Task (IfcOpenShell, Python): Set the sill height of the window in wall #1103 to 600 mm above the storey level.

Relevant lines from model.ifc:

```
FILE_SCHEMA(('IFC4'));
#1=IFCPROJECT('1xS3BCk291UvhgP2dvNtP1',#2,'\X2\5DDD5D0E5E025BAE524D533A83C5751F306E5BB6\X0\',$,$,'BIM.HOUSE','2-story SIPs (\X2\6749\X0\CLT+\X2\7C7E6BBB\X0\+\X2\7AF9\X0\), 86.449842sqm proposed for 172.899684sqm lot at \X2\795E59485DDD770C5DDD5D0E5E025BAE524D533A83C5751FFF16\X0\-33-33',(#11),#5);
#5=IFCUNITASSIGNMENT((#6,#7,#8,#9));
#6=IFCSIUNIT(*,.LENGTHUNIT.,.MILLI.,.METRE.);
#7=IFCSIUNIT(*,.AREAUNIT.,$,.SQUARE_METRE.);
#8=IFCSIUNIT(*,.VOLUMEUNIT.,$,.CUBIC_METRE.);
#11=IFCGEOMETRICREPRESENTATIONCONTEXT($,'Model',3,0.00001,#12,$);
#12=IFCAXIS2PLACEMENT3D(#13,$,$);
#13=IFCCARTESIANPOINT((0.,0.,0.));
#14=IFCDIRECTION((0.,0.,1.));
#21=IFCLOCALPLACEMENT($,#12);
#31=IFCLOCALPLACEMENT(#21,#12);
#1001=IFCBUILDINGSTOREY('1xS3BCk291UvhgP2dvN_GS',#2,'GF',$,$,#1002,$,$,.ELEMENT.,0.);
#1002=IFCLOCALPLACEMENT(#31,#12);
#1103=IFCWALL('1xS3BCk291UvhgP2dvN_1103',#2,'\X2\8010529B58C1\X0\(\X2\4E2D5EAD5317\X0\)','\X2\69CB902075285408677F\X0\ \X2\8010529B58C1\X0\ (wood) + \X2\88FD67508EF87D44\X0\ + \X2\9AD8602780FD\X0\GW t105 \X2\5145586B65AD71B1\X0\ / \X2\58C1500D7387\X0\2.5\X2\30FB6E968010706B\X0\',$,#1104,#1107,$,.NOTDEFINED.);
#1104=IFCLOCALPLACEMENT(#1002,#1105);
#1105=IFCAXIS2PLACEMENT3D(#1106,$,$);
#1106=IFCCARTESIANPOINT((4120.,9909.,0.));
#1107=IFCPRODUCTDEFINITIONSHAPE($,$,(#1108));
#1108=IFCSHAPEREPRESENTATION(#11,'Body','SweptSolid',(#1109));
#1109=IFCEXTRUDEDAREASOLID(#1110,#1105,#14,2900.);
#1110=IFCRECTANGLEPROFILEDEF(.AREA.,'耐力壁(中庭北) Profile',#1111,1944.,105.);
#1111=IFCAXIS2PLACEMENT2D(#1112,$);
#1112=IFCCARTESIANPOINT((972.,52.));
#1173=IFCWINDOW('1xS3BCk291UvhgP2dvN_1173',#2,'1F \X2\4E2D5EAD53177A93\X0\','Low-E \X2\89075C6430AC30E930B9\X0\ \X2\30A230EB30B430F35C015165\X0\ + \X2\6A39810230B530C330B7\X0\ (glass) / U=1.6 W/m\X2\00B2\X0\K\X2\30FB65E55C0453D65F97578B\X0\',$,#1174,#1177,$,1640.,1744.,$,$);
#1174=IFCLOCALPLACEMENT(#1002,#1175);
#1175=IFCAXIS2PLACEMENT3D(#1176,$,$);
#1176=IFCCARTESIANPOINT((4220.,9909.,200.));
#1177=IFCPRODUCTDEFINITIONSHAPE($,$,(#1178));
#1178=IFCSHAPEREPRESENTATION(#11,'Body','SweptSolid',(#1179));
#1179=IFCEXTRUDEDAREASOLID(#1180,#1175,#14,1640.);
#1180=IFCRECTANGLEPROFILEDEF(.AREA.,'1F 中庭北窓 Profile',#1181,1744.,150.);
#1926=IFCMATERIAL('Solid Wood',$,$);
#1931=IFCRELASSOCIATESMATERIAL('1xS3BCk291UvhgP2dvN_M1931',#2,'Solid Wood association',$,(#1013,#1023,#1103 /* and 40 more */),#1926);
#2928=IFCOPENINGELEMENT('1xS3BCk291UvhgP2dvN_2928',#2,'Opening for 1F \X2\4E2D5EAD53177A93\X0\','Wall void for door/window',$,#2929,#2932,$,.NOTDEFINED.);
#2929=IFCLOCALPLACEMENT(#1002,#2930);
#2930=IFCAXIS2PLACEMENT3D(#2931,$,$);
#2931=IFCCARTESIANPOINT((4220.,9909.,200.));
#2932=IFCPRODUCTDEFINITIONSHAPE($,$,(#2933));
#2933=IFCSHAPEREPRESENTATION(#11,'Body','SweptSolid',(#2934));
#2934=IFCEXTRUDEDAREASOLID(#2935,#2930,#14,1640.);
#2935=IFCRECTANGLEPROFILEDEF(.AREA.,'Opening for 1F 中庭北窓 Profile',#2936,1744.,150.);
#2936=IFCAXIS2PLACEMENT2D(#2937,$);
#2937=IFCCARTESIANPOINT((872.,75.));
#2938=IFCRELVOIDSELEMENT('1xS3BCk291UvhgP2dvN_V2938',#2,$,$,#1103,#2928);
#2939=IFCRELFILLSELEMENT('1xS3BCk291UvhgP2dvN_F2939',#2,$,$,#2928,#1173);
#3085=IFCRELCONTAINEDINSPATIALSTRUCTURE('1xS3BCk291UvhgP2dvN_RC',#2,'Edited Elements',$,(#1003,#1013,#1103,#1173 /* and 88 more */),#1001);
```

```python
import numpy as np
import ifcopenshell
import ifcopenshell.api.geometry
import ifcopenshell.geom
import ifcopenshell.util.element
import ifcopenshell.util.placement
import ifcopenshell.util.shape
import ifcopenshell.util.unit

model = ifcopenshell.open("model.ifc")
unit_scale = ifcopenshell.util.unit.calculate_unit_scale(model)

window = model.by_guid("1xS3BCk291UvhgP2dvN_1173")
opening = window.FillsVoids[0].RelatingOpeningElement
storey = ifcopenshell.util.element.get_container(window, ifc_class="IfcBuildingStorey")
level = ifcopenshell.util.placement.get_local_placement(storey.ObjectPlacement)[2, 3]

# The opening's origin need not be at the sill, so measure its lowest point.
shape = ifcopenshell.geom.create_shape(ifcopenshell.geom.settings(), opening)
bottom = ifcopenshell.util.shape.get_shape_bottom_elevation(shape, shape.geometry) / unit_scale
dz = level + 600.0 - bottom

shift = np.array([0.0, 0.0, dz])
# The window is not placed relative to its opening, so move both.
for product in (opening, window):
    matrix = ifcopenshell.util.placement.get_local_placement(product.ObjectPlacement)
    matrix[:3, 3] += shift
    ifcopenshell.api.geometry.edit_object_placement(model, product=product, matrix=matrix, is_si=False)

print(f"moved by {dz * unit_scale:+.3f} m")

model.write("model_edited.ifc")
```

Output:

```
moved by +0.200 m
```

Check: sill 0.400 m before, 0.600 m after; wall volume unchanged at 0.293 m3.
